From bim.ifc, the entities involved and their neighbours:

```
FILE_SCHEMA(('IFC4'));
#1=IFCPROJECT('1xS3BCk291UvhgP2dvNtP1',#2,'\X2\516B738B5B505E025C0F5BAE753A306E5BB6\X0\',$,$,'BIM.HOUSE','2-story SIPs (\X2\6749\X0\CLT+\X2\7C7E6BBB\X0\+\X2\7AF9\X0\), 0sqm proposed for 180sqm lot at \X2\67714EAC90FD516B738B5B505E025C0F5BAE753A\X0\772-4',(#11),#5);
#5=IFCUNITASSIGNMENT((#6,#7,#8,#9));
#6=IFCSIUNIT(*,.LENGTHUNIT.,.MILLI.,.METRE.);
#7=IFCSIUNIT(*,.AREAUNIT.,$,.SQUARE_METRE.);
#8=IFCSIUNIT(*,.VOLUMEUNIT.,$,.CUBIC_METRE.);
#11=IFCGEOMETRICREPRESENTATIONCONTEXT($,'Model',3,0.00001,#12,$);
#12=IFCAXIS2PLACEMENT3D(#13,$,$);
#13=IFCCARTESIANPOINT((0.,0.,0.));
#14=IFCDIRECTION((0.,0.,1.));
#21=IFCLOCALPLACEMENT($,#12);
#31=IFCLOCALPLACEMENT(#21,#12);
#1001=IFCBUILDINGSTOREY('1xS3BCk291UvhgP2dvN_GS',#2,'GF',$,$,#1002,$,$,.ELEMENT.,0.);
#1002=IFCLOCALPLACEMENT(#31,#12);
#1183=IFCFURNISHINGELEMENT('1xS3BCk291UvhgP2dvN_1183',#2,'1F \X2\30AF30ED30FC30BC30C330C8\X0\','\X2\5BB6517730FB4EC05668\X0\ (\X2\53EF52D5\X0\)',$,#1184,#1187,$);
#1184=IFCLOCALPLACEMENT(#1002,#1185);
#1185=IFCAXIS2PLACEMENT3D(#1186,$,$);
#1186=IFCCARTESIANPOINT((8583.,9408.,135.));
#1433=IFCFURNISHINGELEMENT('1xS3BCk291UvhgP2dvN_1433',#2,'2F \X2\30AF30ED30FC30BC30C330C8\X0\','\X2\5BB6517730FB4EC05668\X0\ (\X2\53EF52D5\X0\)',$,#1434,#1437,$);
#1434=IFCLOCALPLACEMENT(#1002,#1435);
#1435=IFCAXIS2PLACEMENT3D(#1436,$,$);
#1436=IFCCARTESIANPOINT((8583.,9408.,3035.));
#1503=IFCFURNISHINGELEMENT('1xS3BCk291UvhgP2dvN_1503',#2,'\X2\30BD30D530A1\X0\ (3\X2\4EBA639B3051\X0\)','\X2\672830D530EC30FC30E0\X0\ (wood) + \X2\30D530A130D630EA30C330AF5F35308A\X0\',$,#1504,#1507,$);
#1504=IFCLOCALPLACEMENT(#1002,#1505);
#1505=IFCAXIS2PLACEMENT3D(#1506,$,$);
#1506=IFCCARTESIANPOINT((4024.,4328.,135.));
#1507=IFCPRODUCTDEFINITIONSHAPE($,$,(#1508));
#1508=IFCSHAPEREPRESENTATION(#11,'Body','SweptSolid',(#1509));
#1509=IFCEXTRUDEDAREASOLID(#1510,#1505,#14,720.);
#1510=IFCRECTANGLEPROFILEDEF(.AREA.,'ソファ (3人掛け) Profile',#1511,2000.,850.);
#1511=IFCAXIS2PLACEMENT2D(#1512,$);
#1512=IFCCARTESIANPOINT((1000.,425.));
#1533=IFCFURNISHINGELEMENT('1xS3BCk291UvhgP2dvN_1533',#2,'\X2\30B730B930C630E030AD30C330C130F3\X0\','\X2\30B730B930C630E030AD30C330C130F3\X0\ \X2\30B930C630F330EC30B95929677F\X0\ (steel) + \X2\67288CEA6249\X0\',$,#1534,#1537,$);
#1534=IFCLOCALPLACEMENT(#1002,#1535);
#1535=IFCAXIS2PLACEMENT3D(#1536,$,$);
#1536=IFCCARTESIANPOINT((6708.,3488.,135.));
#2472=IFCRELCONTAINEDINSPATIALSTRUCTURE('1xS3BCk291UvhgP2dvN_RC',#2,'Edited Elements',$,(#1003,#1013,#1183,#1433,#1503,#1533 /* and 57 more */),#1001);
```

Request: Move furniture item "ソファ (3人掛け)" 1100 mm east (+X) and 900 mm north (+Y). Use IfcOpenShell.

```python
import ifcopenshell
import ifcopenshell.api.geometry
import ifcopenshell.util.placement

model = ifcopenshell.open("bim.ifc")

item = model.by_guid("1xS3BCk291UvhgP2dvN_1503")
matrix = ifcopenshell.util.placement.get_local_placement(item.ObjectPlacement)
matrix[0, 3] += 1100.0
matrix[1, 3] += 900.0
ifcopenshell.api.geometry.edit_object_placement(model, product=item, matrix=matrix, is_si=False)

print(ifcopenshell.util.placement.get_local_placement(item.ObjectPlacement).round(3) + 0.0)

model.write("bim_v2.ifc")
```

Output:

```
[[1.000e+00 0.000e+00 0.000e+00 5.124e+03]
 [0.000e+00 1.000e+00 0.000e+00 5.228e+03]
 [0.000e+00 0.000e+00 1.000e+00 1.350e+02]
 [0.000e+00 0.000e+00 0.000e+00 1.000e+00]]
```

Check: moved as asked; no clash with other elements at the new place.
